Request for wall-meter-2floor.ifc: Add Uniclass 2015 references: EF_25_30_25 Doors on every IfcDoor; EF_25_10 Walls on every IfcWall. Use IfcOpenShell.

First a look at what the model holds.

```python
import ifcopenshell

model = ifcopenshell.open("wall-meter-2floor.ifc")
print(model.schema)
print("classifications:", [c.Name for c in model.by_type("IfcClassification")])
for ifc_class in ("IfcDoor", "IfcRoof", "IfcStair", "IfcWall", "IfcWindow"):
    print(ifc_class, len(model.by_type(ifc_class)))
```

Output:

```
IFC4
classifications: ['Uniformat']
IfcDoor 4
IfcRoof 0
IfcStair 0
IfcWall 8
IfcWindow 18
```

```python
import ifcopenshell
import ifcopenshell.api.classification

model = ifcopenshell.open("wall-meter-2floor.ifc")

system = ifcopenshell.api.classification.add_classification(model, classification="Uniclass 2015")

codes = {
    "IfcDoor": ("EF_25_30_25", "Doors"),
    "IfcWall": ("EF_25_10", "Walls"),
}
for ifc_class, (code, name) in codes.items():
    products = model.by_type(ifc_class)
    ifcopenshell.api.classification.add_reference(
        model, products=products, classification=system, identification=code, name=name
    )
    print(code, len(products))

model.write("wall-meter-2floor_v2.ifc")
```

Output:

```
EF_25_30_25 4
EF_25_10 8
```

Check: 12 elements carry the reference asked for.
